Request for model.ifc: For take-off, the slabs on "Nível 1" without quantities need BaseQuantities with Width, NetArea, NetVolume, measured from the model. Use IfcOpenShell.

First a look at what the model holds.

```python
import ifcopenshell
import ifcopenshell.util.element
import ifcopenshell.util.unit

model = ifcopenshell.open("model.ifc")
print(model.schema)
for unit_type in ("LENGTHUNIT", "AREAUNIT", "VOLUMEUNIT"):
    print(unit_type, ifcopenshell.util.unit.calculate_unit_scale(model, unit_type))
storey = next(s for s in model.by_type("IfcBuildingStorey") if s.Name == "Nível 1")
slabs = [e for e in ifcopenshell.util.element.get_decomposition(storey) if e.is_a("IfcSlab")]
for e in sorted(slabs, key=lambda e: e.id()):
    print(e.id(), e.is_a(), e.Name, list(ifcopenshell.util.element.get_psets(e, qtos_only=True)), sep=" | ")
```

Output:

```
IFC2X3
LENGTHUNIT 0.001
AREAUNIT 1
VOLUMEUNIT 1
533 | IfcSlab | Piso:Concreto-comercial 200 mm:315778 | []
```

```python
import ifcopenshell
import ifcopenshell.api.pset
import ifcopenshell.geom
import ifcopenshell.util.element
import ifcopenshell.util.shape
import ifcopenshell.util.unit

model = ifcopenshell.open("model.ifc")
unit_scale = ifcopenshell.util.unit.calculate_unit_scale(model)
area_scale = ifcopenshell.util.unit.calculate_unit_scale(model, "AREAUNIT")
volume_scale = ifcopenshell.util.unit.calculate_unit_scale(model, "VOLUMEUNIT")
settings = ifcopenshell.geom.settings()

storey = next(s for s in model.by_type("IfcBuildingStorey") if s.Name == "Nível 1")
slabs = [e for e in ifcopenshell.util.element.get_decomposition(storey) if e.is_a("IfcSlab")]

for e in sorted(slabs, key=lambda e: e.id()):
    if ifcopenshell.util.element.get_psets(e, qtos_only=True, should_inherit=False):
        continue
    # Geometry comes back in metres, in the element's own axes.
    shape = ifcopenshell.geom.create_shape(settings, e)
    values = {
        "Width": ifcopenshell.util.shape.get_z(shape.geometry) / unit_scale,
        "NetArea": ifcopenshell.util.shape.get_footprint_area(shape.geometry) / area_scale,
        "NetVolume": ifcopenshell.util.shape.get_volume(shape.geometry) / volume_scale,
    }
    qto = ifcopenshell.api.pset.add_qto(model, product=e, name="BaseQuantities")
    ifcopenshell.api.pset.edit_qto(model, qto=qto, properties=values)
    print(e.id(), {k: round(v, 3) for k, v in values.items()})

model.write("model_rev.ifc")
```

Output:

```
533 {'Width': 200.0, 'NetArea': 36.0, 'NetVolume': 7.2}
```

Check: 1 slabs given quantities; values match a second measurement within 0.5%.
